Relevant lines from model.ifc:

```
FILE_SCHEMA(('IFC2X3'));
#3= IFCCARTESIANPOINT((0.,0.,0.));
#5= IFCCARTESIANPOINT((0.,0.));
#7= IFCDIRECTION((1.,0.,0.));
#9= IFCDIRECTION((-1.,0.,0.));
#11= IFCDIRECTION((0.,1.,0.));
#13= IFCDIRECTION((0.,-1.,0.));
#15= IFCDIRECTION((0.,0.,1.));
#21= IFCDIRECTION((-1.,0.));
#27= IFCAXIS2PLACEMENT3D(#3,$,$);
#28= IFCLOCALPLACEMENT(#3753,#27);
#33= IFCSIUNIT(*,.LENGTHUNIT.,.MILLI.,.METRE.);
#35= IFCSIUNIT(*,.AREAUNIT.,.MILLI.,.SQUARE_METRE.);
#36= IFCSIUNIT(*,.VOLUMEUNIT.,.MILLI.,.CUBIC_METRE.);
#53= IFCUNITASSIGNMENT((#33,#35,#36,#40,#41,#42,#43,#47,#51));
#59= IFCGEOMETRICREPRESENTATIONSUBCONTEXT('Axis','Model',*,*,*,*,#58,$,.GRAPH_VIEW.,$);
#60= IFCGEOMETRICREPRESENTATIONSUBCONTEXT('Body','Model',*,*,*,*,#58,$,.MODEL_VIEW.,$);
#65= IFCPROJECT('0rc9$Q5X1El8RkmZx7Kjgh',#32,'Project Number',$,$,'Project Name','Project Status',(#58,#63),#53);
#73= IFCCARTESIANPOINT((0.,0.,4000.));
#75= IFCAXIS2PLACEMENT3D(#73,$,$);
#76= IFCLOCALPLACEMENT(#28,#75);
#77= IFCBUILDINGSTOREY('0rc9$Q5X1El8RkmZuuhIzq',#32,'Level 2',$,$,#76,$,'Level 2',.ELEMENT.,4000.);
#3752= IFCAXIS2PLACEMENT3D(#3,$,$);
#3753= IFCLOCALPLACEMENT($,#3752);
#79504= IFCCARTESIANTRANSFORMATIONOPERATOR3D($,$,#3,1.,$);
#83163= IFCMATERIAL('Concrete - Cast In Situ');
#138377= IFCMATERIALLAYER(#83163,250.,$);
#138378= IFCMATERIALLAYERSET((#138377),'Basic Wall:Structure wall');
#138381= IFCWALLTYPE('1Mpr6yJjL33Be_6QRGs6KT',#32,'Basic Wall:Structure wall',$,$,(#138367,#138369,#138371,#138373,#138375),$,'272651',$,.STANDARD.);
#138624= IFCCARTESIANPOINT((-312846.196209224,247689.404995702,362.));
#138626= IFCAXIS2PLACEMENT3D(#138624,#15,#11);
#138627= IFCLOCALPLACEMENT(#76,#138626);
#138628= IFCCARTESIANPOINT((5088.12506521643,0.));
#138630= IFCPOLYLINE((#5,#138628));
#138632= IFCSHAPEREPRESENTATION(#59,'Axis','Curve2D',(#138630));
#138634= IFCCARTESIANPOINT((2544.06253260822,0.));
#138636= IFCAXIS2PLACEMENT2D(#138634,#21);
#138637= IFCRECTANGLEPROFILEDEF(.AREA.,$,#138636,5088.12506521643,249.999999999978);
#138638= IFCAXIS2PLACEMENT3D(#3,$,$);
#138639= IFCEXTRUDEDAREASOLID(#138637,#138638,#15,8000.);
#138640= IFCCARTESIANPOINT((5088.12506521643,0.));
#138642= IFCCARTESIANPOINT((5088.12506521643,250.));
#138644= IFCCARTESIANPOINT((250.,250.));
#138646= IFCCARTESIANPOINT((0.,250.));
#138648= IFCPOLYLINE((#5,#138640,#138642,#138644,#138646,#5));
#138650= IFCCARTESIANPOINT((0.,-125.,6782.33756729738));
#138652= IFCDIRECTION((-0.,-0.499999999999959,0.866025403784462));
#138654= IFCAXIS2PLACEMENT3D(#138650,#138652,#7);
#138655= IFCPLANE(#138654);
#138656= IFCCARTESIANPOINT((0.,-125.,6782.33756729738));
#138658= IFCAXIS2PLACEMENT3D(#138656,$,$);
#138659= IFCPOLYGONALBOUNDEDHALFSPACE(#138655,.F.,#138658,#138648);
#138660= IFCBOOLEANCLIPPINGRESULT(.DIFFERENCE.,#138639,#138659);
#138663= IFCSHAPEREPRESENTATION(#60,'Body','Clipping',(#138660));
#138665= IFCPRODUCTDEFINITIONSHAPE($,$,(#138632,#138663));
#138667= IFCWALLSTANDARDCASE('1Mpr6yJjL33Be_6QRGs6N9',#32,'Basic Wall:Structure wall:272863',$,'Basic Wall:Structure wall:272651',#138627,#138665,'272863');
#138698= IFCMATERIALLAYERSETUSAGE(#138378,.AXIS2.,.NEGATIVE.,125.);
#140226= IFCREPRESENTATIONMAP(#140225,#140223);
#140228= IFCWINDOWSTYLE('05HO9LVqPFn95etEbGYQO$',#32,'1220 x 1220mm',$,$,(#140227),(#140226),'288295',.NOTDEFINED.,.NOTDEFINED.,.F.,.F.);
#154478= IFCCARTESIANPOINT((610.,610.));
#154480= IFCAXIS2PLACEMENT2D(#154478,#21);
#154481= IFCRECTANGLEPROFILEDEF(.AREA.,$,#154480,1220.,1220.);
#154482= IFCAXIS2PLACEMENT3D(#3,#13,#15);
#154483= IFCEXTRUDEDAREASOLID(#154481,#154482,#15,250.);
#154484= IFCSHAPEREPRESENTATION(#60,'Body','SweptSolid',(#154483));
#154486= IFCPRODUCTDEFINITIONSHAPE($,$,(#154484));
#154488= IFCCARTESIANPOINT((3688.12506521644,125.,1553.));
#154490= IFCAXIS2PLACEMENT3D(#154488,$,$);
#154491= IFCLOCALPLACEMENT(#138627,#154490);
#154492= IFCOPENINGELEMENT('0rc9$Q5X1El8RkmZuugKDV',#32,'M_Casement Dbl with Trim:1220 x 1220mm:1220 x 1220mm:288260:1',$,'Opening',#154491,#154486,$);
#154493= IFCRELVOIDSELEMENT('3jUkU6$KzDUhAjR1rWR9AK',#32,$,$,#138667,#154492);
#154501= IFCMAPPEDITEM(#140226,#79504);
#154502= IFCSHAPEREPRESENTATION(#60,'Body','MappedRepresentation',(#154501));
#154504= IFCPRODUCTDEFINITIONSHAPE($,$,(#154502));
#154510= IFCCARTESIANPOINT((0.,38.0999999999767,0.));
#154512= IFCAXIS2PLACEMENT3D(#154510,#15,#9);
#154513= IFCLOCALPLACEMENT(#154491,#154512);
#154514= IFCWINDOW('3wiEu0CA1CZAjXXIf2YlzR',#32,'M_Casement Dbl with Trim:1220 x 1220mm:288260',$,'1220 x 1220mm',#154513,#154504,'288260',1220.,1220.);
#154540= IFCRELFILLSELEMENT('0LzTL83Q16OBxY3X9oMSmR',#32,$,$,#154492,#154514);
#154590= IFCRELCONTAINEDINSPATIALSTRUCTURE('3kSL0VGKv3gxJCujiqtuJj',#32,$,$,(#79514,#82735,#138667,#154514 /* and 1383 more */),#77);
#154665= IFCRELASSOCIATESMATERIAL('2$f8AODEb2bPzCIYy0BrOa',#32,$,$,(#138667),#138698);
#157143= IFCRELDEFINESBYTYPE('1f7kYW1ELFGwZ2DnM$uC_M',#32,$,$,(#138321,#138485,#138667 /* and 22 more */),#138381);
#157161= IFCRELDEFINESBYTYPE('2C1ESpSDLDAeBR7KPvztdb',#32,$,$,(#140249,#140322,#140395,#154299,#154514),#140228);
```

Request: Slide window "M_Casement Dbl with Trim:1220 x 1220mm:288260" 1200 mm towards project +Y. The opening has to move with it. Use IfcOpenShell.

```python
import ifcopenshell
import ifcopenshell.api.geometry
import ifcopenshell.util.placement

model = ifcopenshell.open("model.ifc")

window = model.by_guid("3wiEu0CA1CZAjXXIf2YlzR")
opening = window.FillsVoids[0].RelatingOpeningElement
wall = opening.VoidsElements[0].RelatingBuildingElement

wall_matrix = ifcopenshell.util.placement.get_local_placement(wall.ObjectPlacement)
shift = wall_matrix[:3, 0] * 1200.0
before = ifcopenshell.util.placement.get_local_placement(window.ObjectPlacement)[:3, 3].copy()

# The window is placed relative to its opening, so it follows when the opening moves.
matrix = ifcopenshell.util.placement.get_local_placement(opening.ObjectPlacement)
matrix[:3, 3] += shift
ifcopenshell.api.geometry.edit_object_placement(
    model, product=opening, matrix=matrix, is_si=False, should_transform_children=True
)

after = ifcopenshell.util.placement.get_local_placement(window.ObjectPlacement)[:3, 3]
print("window moved by", (after - before).round(3) + 0.0)

model.write("model_rev.ifc")
```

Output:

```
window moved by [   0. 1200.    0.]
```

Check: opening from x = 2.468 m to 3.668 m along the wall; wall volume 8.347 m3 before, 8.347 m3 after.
